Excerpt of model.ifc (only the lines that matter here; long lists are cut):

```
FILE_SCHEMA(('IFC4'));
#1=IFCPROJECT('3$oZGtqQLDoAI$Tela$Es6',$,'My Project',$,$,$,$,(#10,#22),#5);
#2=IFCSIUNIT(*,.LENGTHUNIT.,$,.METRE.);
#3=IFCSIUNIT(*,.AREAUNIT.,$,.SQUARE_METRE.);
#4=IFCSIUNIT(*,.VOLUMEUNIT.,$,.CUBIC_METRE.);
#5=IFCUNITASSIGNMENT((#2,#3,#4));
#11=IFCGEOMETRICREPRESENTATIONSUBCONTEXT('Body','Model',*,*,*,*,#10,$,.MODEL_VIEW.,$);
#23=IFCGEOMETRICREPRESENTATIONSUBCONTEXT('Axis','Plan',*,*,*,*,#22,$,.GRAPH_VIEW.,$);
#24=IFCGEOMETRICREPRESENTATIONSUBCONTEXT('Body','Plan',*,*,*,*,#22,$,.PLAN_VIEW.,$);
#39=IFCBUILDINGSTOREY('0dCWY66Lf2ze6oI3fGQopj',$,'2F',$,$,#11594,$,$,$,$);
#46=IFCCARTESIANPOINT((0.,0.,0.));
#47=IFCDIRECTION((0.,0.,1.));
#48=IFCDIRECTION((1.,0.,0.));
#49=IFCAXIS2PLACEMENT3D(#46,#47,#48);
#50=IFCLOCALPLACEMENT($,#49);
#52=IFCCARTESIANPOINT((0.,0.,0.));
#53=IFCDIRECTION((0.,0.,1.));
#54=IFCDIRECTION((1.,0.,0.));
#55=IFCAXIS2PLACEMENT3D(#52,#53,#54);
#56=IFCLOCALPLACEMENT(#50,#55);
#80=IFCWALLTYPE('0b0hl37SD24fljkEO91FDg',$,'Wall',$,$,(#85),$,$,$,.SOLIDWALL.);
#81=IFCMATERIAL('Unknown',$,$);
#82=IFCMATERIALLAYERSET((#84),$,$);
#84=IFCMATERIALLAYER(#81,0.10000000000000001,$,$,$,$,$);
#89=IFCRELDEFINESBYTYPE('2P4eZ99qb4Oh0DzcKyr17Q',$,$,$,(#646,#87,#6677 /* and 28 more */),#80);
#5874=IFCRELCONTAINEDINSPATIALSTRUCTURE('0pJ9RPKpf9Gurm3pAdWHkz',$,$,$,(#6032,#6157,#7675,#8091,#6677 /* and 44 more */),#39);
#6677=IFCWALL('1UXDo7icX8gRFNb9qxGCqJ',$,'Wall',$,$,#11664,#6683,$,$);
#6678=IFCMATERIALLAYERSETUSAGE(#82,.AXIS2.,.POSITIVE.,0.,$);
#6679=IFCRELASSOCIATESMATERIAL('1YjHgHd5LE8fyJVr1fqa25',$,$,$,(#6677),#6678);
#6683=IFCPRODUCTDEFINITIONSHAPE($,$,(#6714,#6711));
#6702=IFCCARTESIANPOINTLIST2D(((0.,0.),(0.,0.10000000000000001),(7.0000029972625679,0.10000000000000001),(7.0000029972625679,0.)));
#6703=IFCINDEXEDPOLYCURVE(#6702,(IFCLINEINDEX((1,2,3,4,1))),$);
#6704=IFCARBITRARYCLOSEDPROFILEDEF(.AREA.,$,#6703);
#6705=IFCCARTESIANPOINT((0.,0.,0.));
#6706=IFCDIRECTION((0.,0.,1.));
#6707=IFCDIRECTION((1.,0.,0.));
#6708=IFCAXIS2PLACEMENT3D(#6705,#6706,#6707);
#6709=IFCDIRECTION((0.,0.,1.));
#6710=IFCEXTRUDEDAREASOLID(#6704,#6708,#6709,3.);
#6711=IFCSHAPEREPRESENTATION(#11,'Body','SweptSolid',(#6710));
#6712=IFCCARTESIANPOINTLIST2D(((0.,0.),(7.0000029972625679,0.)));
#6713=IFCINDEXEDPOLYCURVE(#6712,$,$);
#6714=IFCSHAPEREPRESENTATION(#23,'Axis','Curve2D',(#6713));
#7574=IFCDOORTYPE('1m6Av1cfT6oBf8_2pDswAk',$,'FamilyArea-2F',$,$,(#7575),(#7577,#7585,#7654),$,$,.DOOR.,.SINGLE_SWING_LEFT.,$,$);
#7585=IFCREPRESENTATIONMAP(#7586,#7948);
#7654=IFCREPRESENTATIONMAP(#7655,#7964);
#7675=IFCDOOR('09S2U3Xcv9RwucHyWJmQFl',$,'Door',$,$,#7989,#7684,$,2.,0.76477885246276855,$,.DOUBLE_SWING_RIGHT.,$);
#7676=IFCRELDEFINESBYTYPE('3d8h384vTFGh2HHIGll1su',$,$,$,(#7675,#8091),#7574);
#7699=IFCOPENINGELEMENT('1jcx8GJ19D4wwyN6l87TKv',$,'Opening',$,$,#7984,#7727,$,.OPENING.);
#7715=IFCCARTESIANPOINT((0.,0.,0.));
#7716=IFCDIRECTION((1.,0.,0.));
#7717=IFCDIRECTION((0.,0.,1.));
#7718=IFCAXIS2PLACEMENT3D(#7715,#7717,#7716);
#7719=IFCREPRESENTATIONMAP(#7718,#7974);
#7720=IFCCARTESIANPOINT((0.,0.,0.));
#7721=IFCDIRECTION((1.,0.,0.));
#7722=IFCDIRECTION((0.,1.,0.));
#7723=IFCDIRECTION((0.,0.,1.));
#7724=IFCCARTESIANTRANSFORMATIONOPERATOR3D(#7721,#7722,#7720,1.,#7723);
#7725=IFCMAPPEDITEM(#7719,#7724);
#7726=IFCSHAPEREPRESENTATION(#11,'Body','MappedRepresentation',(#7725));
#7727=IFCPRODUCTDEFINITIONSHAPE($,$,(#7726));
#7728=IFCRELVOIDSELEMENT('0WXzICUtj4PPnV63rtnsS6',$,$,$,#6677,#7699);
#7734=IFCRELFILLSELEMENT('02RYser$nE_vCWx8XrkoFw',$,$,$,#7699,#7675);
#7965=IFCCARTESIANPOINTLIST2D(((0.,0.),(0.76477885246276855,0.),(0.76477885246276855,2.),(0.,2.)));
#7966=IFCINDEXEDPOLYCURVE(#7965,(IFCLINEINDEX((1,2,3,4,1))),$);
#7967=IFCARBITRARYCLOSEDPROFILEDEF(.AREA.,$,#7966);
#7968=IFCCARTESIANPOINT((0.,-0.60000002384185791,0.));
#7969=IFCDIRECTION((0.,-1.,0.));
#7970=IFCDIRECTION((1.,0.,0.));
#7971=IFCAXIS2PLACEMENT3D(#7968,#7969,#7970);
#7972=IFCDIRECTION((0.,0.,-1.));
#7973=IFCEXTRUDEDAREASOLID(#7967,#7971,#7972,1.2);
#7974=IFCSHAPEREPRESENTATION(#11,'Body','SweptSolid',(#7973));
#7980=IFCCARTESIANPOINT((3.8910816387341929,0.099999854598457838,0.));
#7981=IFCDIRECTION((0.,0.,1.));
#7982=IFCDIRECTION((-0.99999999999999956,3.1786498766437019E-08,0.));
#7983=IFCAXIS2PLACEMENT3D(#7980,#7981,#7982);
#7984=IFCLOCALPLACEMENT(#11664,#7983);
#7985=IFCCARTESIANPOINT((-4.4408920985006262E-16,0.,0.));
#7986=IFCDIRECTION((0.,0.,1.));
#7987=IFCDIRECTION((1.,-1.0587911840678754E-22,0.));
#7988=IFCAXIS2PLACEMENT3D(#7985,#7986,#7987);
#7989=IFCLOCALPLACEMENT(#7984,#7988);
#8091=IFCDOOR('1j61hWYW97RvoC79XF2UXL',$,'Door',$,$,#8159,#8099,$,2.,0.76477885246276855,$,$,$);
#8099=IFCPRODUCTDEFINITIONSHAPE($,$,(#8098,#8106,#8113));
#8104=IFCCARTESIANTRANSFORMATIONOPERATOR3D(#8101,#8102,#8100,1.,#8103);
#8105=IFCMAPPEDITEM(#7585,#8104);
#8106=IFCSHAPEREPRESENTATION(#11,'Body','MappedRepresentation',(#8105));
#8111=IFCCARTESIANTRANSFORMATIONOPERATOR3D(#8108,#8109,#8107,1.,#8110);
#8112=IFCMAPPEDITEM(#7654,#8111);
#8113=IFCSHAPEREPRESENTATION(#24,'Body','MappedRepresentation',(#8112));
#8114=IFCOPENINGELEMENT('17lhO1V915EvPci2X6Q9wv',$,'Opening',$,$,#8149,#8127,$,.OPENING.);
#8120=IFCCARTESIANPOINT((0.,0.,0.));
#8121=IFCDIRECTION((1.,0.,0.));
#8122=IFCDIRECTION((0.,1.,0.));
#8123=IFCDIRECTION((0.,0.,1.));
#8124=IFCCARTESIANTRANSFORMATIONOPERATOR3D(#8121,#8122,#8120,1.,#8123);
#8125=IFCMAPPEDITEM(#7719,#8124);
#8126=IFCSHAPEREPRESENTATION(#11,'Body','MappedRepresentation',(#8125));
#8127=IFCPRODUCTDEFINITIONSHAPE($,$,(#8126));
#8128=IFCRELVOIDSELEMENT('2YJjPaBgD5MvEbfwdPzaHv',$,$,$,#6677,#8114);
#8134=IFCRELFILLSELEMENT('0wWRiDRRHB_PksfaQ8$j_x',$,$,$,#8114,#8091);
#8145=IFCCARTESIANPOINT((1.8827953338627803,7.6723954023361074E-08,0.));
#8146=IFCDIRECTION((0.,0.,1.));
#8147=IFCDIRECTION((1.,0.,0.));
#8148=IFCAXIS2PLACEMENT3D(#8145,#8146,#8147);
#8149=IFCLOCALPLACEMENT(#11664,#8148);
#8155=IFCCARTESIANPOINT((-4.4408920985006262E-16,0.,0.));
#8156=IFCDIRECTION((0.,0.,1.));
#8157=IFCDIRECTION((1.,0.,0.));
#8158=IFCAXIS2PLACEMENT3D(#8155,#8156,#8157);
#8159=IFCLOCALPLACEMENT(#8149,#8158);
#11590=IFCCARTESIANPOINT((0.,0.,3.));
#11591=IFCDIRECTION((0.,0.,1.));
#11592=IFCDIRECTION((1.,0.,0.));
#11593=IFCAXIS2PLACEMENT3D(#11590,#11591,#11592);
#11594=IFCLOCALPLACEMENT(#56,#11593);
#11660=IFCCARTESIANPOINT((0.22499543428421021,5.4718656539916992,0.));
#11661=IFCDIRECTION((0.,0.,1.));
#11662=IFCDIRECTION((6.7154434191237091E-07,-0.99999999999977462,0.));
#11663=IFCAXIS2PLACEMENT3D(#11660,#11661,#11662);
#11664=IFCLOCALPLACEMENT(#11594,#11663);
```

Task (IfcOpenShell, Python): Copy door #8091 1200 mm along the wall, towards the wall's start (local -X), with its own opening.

```python
import ifcopenshell
import ifcopenshell.api.feature
import ifcopenshell.api.geometry
import ifcopenshell.api.root
import ifcopenshell.geom
import ifcopenshell.util.element
import ifcopenshell.util.placement
import ifcopenshell.util.shape
import ifcopenshell.util.unit

model = ifcopenshell.open("model.ifc")
unit_scale = ifcopenshell.util.unit.calculate_unit_scale(model)
settings = ifcopenshell.geom.settings()


def volume(element):
    """Net volume in cubic metres, openings subtracted."""
    shape = ifcopenshell.geom.create_shape(settings, element)
    return ifcopenshell.util.shape.get_volume(shape.geometry)


door = model.by_guid("1j61hWYW97RvoC79XF2UXL")
opening = door.FillsVoids[0].RelatingOpeningElement
wall = opening.VoidsElements[0].RelatingBuildingElement
before = volume(wall)
shift = ifcopenshell.util.placement.get_local_placement(wall.ObjectPlacement)[:3, 0] * -1.2 / unit_scale

# copy_class copies the void relationship, type, container and properties, but no geometry.
new_opening = ifcopenshell.api.root.copy_class(model, product=opening)
new_opening.Representation = ifcopenshell.util.element.copy_deep(
    model, opening.Representation, exclude=["IfcGeometricRepresentationContext", "IfcRepresentationMap"]
)
new_door = ifcopenshell.api.root.copy_class(model, product=door)
new_door.Representation = ifcopenshell.util.element.copy_deep(
    model, door.Representation, exclude=["IfcGeometricRepresentationContext", "IfcRepresentationMap"]
)
ifcopenshell.api.feature.add_filling(model, opening=new_opening, element=new_door)

for old, new in ((opening, new_opening), (door, new_door)):
    matrix = ifcopenshell.util.placement.get_local_placement(old.ObjectPlacement)
    matrix[:3, 3] += shift
    ifcopenshell.api.geometry.edit_object_placement(model, product=new, matrix=matrix, is_si=False)

after = volume(wall)

print(f"wall volume {before:.3f} -> {after:.3f} m3")

model.write("model_updated.ifc")
```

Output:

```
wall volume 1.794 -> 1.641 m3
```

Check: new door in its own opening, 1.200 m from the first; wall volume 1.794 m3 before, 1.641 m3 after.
